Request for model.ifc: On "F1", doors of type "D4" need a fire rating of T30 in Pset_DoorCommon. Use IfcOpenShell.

First a look at what the model holds.

```python
import ifcopenshell
import ifcopenshell.util.element

model = ifcopenshell.open("model.ifc")
print(model.schema)
storey = next(s for s in model.by_type("IfcBuildingStorey") if s.Name == "F1")
doors = [e for e in ifcopenshell.util.element.get_decomposition(storey) if e.is_a("IfcDoor")]
seen = {}
for e in doors:
    element_type = ifcopenshell.util.element.get_type(e)
    key = (element_type.Name if element_type != e and element_type else None, ifcopenshell.util.element.get_pset(e, "Pset_DoorCommon", "FireRating"))
    seen[key] = seen.get(key, 0) + 1
for (name, value), count in sorted(seen.items(), key=str):
    print(count, "x", name, "|", value)
```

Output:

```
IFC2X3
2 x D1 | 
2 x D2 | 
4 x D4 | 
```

```python
import ifcopenshell
import ifcopenshell.api.pset
import ifcopenshell.util.element

model = ifcopenshell.open("model.ifc")

storey = next(s for s in model.by_type("IfcBuildingStorey") if s.Name == "F1")
doors = [e for e in ifcopenshell.util.element.get_decomposition(storey) if e.is_a("IfcDoor")]

count = 0
for e in doors:
    element_type = ifcopenshell.util.element.get_type(e)
    if element_type in (None, e) or element_type.Name != "D4":
        continue
    # add_pset returns the element's existing set when there is one.
    pset = ifcopenshell.api.pset.add_pset(model, product=e, name="Pset_DoorCommon")
    ifcopenshell.api.pset.edit_pset(model, pset=pset, properties={"FireRating": "T30"})
    count += 1

print(count, "doors updated")

model.write("model-out.ifc")
```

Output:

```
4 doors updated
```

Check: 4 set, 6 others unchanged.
